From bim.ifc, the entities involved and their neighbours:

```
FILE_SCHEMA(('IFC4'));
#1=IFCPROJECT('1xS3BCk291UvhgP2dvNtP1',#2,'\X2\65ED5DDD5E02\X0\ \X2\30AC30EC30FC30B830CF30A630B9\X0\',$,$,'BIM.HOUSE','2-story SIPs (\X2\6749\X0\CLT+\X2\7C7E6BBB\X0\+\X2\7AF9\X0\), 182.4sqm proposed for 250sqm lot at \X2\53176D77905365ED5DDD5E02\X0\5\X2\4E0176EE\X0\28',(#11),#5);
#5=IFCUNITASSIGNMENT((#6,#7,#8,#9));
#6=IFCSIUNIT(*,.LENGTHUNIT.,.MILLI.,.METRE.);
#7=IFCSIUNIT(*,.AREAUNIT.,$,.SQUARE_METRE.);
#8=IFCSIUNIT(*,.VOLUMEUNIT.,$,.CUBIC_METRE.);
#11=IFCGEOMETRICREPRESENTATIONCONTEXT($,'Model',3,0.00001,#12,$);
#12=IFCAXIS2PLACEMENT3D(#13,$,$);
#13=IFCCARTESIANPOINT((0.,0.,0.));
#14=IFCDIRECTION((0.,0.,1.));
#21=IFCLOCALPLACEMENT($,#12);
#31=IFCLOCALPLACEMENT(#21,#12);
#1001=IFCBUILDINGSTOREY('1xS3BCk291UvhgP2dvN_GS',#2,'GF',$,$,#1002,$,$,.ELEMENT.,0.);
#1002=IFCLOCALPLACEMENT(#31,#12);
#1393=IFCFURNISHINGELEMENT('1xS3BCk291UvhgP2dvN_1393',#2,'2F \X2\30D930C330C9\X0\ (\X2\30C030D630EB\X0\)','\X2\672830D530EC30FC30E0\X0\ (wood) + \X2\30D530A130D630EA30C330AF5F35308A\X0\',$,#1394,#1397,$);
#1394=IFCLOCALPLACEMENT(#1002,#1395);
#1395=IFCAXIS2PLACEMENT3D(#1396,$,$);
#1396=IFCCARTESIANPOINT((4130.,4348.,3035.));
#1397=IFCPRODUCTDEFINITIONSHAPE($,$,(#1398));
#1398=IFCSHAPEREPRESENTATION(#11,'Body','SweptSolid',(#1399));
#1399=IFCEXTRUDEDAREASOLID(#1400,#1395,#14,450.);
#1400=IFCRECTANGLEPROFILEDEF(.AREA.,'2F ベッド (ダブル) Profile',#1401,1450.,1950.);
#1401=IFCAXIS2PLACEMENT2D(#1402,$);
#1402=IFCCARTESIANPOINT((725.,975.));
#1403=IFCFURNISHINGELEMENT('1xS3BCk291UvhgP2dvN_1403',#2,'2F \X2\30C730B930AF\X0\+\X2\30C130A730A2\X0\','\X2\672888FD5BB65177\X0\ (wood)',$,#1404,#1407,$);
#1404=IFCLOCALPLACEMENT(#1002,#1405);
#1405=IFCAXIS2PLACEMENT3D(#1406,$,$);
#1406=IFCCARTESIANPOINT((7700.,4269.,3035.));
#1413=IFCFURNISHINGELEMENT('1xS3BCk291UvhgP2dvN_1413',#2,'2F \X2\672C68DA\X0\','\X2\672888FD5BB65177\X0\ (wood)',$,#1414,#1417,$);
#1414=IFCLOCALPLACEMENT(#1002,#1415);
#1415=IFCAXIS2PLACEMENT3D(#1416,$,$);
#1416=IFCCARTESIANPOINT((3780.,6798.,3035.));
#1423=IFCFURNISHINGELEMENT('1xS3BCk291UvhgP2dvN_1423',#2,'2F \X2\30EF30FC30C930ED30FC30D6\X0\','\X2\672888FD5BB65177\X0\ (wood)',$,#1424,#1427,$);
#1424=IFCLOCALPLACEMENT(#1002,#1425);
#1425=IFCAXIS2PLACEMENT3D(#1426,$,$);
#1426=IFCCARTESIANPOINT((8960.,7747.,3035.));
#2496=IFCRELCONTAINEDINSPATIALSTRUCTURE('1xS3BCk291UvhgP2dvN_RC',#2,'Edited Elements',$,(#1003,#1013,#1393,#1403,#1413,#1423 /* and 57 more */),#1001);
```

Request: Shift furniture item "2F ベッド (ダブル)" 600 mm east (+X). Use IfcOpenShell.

```python
import ifcopenshell
import ifcopenshell.api.geometry
import ifcopenshell.util.placement
import ifcopenshell.util.unit

model = ifcopenshell.open("bim.ifc")
unit_scale = ifcopenshell.util.unit.calculate_unit_scale(model)

item = model.by_guid("1xS3BCk291UvhgP2dvN_1393")
matrix = ifcopenshell.util.placement.get_local_placement(item.ObjectPlacement)
matrix[0, 3] += 0.6 / unit_scale
ifcopenshell.api.geometry.edit_object_placement(model, product=item, matrix=matrix, is_si=False)

print(ifcopenshell.util.placement.get_local_placement(item.ObjectPlacement).round(3) + 0.0)

model.write("bim_updated.ifc")
```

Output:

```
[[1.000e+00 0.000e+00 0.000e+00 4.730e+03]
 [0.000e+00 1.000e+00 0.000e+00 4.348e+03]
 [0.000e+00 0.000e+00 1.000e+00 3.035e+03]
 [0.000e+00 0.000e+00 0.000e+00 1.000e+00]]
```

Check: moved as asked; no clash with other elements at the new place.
